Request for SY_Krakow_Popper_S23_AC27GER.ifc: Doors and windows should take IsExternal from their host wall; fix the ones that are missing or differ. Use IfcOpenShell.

First a look at what the model holds.

```python
import ifcopenshell
import ifcopenshell.util.element

model = ifcopenshell.open("SY_Krakow_Popper_S23_AC27GER.ifc")
print(model.schema)
seen = {}
for e in model.by_type("IfcDoor") + model.by_type("IfcWindow"):
    if not e.FillsVoids:
        continue
    host = e.FillsVoids[0].RelatingOpeningElement.VoidsElements[0].RelatingBuildingElement
    own = ifcopenshell.util.element.get_pset(e, f"Pset_{e.is_a()[3:].removesuffix('StandardCase')}Common", "IsExternal")
    wall = ifcopenshell.util.element.get_pset(host, "Pset_WallCommon", "IsExternal")
    seen[e.is_a(), own, wall] = seen.get((e.is_a(), own, wall), 0) + 1
for (cls, own, wall), count in sorted(seen.items(), key=str):
    print(count, cls, "IsExternal:", own, "| host wall:", wall)
```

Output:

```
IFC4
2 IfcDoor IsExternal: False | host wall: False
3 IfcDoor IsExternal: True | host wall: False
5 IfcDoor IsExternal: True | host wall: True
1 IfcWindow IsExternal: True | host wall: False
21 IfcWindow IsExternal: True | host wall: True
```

```python
import ifcopenshell
import ifcopenshell.api.pset
import ifcopenshell.util.element

model = ifcopenshell.open("SY_Krakow_Popper_S23_AC27GER.ifc")

count = 0
for ifc_class, pset_name in (("IfcDoor", "Pset_DoorCommon"), ("IfcWindow", "Pset_WindowCommon")):
    for e in model.by_type(ifc_class):
        if not e.FillsVoids:
            continue
        host = e.FillsVoids[0].RelatingOpeningElement.VoidsElements[0].RelatingBuildingElement
        external = ifcopenshell.util.element.get_pset(host, "Pset_WallCommon", "IsExternal")
        if external is None or ifcopenshell.util.element.get_pset(e, pset_name, "IsExternal") == external:
            continue
        pset = ifcopenshell.api.pset.add_pset(model, product=e, name=pset_name)
        ifcopenshell.api.pset.edit_pset(model, pset=pset, properties={"IsExternal": external})
        count += 1

print(count, "updated")

model.write("SY_Krakow_Popper_S23_AC27GER-out.ifc")
```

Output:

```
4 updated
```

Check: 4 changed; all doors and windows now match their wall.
